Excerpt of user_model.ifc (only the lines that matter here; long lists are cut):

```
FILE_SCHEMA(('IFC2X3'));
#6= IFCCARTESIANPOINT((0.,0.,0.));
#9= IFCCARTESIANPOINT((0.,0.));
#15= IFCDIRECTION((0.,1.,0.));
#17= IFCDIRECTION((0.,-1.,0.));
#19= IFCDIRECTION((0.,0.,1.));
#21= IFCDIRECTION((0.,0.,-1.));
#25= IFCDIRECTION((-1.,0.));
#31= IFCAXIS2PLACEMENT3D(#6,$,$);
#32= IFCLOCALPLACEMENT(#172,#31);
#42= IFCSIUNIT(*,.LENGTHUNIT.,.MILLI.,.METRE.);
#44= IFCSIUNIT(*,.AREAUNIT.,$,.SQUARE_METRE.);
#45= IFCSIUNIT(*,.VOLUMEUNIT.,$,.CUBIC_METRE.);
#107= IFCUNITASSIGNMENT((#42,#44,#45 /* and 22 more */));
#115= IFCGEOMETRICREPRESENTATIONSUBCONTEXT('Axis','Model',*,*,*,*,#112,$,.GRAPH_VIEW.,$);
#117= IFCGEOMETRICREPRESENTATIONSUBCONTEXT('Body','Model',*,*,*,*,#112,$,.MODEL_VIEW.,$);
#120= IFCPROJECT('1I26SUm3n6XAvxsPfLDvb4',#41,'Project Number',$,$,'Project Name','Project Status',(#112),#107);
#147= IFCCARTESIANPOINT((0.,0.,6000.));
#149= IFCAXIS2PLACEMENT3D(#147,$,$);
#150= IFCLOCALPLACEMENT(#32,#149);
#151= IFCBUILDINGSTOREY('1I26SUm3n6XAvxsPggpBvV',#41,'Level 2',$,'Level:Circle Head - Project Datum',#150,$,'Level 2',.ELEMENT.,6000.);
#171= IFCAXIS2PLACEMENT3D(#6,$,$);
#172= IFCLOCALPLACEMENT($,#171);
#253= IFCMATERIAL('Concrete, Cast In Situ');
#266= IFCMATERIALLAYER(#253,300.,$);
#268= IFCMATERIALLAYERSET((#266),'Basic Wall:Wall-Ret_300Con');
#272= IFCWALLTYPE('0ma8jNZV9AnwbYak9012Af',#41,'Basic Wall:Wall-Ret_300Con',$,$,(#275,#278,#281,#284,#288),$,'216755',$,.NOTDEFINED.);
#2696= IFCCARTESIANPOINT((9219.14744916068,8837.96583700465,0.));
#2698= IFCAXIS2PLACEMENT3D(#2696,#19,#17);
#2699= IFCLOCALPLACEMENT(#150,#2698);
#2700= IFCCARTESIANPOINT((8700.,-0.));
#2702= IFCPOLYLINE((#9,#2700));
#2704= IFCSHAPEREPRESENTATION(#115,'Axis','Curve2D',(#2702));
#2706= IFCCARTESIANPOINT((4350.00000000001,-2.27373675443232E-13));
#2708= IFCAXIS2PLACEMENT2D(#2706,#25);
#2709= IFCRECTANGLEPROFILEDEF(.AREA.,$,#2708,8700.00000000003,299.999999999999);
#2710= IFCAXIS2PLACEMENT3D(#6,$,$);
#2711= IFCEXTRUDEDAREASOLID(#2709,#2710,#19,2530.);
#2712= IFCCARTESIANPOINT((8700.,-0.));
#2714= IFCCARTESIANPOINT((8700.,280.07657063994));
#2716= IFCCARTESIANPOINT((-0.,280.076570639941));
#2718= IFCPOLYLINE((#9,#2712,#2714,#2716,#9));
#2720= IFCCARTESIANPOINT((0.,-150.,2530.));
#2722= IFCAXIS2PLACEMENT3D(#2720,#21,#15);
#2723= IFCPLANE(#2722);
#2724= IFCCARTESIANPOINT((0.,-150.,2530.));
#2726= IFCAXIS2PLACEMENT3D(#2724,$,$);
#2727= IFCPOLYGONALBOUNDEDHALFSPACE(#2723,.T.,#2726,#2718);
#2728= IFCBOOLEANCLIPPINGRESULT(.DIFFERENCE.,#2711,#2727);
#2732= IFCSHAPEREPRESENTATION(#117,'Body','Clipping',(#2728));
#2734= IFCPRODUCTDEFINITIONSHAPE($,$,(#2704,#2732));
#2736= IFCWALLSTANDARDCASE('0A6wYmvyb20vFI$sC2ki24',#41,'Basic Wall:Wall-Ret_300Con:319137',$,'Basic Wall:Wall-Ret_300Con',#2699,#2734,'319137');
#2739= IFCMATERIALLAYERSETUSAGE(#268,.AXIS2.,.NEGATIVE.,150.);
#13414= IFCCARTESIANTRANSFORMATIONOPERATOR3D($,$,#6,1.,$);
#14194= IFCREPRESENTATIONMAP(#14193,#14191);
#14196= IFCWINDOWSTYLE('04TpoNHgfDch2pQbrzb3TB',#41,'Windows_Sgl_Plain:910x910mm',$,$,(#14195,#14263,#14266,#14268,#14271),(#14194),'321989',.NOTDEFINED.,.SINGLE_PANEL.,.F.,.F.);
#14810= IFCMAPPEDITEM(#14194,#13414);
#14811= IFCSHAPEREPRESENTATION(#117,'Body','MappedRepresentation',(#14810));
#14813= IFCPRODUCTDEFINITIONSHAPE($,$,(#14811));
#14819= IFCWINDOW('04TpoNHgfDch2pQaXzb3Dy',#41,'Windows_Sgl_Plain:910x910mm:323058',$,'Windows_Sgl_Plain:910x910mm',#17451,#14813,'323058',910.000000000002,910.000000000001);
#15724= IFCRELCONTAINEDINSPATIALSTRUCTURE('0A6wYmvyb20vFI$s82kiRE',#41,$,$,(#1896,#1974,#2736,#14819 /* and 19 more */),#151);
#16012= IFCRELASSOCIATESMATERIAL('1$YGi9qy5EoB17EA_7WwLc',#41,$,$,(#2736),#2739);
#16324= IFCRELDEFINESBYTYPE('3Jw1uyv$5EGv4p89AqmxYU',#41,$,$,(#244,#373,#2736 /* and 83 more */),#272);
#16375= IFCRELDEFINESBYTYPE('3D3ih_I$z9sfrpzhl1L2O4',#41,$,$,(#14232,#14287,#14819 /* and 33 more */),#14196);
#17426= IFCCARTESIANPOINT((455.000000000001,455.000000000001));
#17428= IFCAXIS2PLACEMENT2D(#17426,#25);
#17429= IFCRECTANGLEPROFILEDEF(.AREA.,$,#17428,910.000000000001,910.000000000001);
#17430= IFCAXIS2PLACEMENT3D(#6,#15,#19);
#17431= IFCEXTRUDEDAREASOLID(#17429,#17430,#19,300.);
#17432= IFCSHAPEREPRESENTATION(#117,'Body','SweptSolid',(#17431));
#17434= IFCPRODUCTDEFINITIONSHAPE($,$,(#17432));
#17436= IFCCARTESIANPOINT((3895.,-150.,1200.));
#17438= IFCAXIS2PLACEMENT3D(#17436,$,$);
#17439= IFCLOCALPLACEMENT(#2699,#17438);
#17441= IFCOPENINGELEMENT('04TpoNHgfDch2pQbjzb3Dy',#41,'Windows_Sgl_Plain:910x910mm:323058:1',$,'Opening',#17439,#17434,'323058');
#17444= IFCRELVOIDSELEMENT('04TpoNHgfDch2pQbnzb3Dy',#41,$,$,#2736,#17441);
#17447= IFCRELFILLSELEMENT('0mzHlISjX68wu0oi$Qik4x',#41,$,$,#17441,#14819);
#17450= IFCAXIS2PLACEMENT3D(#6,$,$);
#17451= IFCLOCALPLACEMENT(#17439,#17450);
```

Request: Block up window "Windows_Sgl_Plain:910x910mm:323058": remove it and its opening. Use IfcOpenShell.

```python
import ifcopenshell
import ifcopenshell.api.feature
import ifcopenshell.api.root
import ifcopenshell.geom
import ifcopenshell.util.shape

model = ifcopenshell.open("user_model.ifc")
settings = ifcopenshell.geom.settings()


def volume(element):
    """Net volume in cubic metres, openings subtracted."""
    shape = ifcopenshell.geom.create_shape(settings, element)
    return ifcopenshell.util.shape.get_volume(shape.geometry)


window = model.by_guid("04TpoNHgfDch2pQaXzb3Dy")
opening = window.FillsVoids[0].RelatingOpeningElement
wall = opening.VoidsElements[0].RelatingBuildingElement
before = volume(wall)

ifcopenshell.api.root.remove_product(model, product=window)
ifcopenshell.api.feature.remove_feature(model, feature=opening)

after = volume(wall)

print(f"wall volume {before:.3f} -> {after:.3f} m3")

model.write("user_model_v2.ifc")
```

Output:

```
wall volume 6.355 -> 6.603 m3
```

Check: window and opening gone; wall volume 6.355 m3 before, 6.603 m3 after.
